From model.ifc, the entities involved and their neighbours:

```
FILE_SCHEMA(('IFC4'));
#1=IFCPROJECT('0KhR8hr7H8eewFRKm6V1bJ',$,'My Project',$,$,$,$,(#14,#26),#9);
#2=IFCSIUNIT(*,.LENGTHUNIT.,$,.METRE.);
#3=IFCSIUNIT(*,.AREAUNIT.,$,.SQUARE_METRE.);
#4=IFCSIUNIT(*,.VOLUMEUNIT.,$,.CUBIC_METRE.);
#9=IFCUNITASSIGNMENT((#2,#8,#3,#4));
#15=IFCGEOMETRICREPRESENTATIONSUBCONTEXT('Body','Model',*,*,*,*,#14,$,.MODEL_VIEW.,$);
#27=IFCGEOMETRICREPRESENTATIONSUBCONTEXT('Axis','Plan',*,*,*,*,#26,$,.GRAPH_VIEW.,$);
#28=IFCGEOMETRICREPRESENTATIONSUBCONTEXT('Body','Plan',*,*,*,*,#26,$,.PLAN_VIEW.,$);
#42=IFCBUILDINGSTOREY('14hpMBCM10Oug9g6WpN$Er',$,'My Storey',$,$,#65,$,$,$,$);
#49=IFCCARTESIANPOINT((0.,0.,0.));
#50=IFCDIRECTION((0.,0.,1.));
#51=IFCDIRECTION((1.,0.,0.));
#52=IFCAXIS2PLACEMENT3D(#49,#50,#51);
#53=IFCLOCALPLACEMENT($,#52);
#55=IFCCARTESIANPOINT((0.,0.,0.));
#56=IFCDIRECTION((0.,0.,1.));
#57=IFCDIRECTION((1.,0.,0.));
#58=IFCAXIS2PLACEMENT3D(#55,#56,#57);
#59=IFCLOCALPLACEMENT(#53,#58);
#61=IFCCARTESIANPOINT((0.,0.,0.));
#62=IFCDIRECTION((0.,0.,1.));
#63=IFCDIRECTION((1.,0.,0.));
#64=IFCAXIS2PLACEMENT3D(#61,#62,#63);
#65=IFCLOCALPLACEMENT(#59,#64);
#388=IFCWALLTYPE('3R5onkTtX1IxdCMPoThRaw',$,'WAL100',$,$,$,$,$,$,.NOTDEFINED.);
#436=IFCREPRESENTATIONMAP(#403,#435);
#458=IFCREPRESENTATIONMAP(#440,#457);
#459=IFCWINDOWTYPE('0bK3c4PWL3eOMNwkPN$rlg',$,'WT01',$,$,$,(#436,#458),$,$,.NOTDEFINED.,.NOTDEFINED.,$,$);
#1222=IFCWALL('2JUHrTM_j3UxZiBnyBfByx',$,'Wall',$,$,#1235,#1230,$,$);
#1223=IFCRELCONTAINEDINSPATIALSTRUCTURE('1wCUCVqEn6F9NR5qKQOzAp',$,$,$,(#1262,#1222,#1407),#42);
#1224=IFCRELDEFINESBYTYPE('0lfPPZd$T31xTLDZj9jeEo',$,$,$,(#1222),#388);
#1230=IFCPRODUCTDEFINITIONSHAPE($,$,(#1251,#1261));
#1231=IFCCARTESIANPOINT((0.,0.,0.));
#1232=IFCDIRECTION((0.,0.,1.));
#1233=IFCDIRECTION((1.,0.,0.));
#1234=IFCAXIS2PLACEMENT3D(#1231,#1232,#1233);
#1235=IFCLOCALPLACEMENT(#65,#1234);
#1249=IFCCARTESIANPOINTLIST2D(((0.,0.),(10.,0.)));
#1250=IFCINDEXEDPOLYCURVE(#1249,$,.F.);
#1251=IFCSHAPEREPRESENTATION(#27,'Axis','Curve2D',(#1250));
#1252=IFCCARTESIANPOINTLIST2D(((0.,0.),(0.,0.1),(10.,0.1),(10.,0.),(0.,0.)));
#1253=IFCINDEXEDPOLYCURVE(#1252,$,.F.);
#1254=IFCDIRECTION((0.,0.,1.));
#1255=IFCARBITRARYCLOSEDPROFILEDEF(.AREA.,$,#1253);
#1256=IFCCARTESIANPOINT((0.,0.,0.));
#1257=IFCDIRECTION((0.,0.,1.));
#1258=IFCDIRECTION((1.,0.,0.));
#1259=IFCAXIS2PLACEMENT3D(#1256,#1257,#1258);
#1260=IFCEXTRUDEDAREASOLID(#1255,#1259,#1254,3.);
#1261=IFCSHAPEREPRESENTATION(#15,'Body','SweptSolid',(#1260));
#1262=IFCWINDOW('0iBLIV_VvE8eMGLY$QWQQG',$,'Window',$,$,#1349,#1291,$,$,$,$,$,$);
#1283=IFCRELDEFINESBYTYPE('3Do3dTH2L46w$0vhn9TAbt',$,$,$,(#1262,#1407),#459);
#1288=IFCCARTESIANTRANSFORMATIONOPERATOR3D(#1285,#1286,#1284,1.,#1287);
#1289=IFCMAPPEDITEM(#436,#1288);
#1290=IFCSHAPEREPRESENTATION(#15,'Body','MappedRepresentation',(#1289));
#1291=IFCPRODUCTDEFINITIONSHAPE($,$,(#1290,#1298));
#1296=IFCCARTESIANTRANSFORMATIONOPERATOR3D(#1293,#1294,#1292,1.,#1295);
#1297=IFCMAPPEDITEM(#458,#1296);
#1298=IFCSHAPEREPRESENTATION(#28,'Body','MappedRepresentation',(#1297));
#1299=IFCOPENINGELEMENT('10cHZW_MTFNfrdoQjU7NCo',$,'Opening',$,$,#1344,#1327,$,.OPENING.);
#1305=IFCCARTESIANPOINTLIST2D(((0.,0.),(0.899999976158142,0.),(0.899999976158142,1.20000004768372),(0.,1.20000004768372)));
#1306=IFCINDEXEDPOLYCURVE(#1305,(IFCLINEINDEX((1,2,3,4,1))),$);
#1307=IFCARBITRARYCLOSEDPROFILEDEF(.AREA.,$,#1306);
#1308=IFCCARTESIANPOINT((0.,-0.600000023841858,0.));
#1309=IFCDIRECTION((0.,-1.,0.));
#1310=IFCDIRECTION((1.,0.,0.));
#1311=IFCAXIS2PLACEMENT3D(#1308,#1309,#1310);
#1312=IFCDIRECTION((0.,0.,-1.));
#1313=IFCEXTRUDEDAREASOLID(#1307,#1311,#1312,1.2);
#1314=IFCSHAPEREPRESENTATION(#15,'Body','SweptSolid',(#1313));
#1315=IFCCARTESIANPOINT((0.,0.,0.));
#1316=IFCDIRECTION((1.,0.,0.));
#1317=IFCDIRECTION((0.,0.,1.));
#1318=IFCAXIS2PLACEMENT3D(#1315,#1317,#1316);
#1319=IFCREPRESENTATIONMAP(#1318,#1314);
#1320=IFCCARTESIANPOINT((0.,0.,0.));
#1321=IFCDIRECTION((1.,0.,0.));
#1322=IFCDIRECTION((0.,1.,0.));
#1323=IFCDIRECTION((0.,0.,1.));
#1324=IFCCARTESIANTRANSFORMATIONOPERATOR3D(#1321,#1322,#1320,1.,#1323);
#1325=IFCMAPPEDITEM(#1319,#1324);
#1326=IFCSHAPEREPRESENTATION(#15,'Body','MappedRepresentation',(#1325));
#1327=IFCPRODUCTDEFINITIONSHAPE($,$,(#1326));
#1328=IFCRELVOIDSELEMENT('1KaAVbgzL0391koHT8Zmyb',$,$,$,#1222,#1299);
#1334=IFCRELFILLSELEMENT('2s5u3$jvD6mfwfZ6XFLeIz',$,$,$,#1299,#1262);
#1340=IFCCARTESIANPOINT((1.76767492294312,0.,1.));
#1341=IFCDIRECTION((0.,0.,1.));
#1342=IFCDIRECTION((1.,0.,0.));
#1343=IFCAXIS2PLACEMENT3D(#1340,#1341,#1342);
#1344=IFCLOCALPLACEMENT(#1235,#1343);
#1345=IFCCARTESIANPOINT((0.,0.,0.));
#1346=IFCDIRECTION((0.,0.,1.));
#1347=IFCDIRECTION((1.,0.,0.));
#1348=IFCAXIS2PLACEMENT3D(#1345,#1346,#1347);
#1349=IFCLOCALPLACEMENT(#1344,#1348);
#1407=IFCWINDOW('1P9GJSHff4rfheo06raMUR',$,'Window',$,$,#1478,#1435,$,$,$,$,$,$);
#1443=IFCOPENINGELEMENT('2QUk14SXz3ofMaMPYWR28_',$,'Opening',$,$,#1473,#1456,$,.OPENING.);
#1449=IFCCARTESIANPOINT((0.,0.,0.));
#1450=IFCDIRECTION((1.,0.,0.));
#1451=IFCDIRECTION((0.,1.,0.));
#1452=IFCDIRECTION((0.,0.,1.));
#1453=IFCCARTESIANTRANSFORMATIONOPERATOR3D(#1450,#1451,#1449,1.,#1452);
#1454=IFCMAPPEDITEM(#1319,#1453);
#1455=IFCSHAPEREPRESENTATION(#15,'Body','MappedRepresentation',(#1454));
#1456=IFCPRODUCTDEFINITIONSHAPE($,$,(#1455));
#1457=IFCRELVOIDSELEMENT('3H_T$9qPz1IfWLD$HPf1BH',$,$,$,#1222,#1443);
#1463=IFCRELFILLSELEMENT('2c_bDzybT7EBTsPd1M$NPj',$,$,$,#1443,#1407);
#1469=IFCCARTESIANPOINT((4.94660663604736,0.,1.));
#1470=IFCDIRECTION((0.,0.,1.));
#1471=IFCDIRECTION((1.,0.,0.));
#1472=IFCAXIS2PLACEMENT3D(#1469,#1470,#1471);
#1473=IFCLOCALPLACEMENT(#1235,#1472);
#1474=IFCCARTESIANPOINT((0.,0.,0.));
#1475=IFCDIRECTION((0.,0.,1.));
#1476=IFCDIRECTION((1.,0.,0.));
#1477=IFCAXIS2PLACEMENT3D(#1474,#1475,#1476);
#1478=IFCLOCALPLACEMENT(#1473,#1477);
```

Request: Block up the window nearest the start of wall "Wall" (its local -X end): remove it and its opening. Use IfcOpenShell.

```python
import ifcopenshell
import ifcopenshell.api.feature
import ifcopenshell.api.root
import ifcopenshell.geom
import ifcopenshell.util.shape

model = ifcopenshell.open("model.ifc")
settings = ifcopenshell.geom.settings()


def volume(element):
    """Net volume in cubic metres, openings subtracted."""
    shape = ifcopenshell.geom.create_shape(settings, element)
    return ifcopenshell.util.shape.get_volume(shape.geometry)


window = model.by_guid("0iBLIV_VvE8eMGLY$QWQQG")
opening = window.FillsVoids[0].RelatingOpeningElement
wall = opening.VoidsElements[0].RelatingBuildingElement
before = volume(wall)

ifcopenshell.api.root.remove_product(model, product=window)
ifcopenshell.api.feature.remove_feature(model, feature=opening)

after = volume(wall)

print(f"wall volume {before:.3f} -> {after:.3f} m3")

model.write("model-out.ifc")
```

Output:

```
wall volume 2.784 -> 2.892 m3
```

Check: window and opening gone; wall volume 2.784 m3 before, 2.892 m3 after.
